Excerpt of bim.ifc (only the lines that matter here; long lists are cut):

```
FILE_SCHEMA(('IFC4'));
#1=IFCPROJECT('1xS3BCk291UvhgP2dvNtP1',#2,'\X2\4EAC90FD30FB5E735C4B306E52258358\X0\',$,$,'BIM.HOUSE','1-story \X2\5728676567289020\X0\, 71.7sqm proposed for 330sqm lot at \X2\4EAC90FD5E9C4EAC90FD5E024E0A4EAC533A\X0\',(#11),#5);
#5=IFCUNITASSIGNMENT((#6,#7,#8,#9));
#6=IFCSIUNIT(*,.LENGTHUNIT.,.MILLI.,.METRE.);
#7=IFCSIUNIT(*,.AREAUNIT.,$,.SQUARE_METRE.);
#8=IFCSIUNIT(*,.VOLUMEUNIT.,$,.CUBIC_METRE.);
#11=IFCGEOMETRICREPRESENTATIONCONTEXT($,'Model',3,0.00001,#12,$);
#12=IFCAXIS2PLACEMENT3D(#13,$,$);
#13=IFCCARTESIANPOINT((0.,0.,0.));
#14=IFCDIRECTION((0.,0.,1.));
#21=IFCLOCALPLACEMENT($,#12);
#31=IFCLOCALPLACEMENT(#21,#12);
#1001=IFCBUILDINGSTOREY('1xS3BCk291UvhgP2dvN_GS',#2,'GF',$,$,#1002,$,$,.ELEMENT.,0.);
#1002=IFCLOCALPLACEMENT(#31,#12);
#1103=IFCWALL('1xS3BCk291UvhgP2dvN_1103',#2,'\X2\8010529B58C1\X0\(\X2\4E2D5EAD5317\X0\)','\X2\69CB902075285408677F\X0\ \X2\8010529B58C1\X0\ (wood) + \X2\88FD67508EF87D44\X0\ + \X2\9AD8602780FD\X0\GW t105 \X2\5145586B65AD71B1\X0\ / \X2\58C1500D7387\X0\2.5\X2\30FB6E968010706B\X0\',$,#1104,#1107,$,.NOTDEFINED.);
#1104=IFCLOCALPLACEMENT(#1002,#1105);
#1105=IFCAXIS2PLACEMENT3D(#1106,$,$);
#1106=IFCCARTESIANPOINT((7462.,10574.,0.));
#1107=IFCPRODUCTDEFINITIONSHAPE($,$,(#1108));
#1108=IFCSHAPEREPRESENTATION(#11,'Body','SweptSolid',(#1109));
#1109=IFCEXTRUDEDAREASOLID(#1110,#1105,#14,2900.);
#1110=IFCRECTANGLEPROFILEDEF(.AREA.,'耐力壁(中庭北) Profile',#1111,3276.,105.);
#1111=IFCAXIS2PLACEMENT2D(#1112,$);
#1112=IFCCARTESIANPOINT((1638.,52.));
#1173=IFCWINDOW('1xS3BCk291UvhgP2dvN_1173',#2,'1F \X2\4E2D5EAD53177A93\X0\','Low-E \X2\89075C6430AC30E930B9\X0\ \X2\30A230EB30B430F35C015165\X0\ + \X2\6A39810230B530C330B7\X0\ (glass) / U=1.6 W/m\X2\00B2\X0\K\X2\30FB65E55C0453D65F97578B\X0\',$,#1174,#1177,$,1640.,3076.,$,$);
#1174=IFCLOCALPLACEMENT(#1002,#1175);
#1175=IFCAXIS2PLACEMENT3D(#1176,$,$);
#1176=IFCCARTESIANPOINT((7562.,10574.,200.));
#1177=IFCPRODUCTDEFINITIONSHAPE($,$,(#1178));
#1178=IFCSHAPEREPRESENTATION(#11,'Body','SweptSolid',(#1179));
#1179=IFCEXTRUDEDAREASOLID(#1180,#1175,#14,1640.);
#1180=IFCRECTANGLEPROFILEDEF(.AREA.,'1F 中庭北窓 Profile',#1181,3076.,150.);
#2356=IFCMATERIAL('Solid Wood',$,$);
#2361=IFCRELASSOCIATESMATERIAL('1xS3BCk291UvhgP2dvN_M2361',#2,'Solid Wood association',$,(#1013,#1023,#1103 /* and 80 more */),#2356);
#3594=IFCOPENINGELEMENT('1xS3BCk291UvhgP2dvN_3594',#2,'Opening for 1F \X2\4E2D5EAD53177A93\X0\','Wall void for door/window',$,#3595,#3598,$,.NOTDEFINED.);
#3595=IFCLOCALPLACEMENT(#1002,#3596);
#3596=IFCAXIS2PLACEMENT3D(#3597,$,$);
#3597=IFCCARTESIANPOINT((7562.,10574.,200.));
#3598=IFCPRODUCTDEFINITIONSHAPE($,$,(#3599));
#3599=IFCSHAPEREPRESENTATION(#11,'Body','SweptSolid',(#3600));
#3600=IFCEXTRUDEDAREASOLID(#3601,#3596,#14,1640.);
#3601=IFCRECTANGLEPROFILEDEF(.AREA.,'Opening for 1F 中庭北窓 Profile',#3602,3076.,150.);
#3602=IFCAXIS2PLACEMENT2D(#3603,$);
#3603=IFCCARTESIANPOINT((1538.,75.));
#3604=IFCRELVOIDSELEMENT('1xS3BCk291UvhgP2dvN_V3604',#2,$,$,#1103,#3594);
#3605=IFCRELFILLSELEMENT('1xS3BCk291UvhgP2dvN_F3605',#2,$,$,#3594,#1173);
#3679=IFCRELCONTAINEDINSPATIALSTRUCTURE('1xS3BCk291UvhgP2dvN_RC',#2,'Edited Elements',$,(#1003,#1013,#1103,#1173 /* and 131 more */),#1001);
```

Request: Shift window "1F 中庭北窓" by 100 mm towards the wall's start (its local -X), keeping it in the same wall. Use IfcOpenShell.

```python
import ifcopenshell
import ifcopenshell.api.geometry
import ifcopenshell.util.placement

model = ifcopenshell.open("bim.ifc")

window = model.by_guid("1xS3BCk291UvhgP2dvN_1173")
opening = window.FillsVoids[0].RelatingOpeningElement
wall = opening.VoidsElements[0].RelatingBuildingElement

wall_matrix = ifcopenshell.util.placement.get_local_placement(wall.ObjectPlacement)
shift = wall_matrix[:3, 0] * -100.0
before = ifcopenshell.util.placement.get_local_placement(window.ObjectPlacement)[:3, 3].copy()

# The window is not placed relative to its opening, so move both.
for product in (opening, window):
    matrix = ifcopenshell.util.placement.get_local_placement(product.ObjectPlacement)
    matrix[:3, 3] += shift
    ifcopenshell.api.geometry.edit_object_placement(model, product=product, matrix=matrix, is_si=False)

after = ifcopenshell.util.placement.get_local_placement(window.ObjectPlacement)[:3, 3]
print("window moved by", (after - before).round(3) + 0.0)

model.write("bim_rev.ifc")
```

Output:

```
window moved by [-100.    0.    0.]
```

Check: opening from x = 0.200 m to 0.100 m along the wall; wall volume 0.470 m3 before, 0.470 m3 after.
